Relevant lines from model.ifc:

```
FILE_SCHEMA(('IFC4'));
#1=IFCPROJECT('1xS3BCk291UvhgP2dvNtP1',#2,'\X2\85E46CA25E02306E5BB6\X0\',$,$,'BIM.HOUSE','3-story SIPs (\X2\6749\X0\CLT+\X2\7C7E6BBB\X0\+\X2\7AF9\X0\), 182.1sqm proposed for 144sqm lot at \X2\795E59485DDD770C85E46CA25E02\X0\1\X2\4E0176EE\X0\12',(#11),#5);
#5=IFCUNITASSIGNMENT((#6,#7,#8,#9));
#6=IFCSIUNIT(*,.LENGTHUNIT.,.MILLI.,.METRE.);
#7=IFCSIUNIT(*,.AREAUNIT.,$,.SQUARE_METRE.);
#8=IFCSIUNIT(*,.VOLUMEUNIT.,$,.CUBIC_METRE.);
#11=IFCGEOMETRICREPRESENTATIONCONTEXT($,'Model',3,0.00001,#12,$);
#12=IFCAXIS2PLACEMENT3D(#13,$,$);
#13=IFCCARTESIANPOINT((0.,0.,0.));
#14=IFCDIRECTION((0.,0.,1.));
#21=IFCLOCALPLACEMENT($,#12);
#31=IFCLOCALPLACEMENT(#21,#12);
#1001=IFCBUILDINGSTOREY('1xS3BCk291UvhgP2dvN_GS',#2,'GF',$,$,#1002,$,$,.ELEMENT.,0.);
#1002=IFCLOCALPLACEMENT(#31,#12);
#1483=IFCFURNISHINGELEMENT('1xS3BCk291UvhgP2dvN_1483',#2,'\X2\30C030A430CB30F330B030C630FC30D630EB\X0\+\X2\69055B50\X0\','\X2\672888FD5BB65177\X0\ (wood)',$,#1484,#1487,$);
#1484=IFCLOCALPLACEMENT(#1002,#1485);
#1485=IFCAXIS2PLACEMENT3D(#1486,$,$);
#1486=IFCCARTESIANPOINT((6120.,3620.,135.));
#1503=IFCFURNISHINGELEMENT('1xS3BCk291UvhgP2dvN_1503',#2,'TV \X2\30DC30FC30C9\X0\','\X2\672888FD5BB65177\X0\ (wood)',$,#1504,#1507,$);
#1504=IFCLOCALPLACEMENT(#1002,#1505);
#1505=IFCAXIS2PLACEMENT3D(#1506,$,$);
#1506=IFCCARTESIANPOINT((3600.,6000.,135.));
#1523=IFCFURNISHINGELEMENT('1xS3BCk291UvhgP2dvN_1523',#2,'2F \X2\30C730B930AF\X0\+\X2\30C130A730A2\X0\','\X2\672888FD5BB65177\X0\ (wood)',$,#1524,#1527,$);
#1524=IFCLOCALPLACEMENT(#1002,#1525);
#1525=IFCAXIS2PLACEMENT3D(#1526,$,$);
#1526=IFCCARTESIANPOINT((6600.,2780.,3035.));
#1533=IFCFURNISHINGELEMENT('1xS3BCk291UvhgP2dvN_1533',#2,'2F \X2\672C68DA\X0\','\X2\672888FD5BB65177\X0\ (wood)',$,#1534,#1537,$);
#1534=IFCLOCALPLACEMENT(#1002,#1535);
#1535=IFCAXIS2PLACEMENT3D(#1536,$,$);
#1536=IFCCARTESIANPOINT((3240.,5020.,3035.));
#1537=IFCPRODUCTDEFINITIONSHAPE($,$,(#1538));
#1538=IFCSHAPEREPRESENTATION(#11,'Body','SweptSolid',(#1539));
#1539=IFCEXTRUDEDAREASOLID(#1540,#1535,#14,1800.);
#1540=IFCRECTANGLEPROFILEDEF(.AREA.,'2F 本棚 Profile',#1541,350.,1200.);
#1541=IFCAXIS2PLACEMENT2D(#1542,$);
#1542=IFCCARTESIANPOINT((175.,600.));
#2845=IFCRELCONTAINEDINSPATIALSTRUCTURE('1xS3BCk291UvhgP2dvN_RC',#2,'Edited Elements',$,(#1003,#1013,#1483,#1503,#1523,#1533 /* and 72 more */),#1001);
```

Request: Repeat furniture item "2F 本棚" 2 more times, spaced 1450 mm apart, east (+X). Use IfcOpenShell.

```python
import numpy as np
import ifcopenshell
import ifcopenshell.api.geometry
import ifcopenshell.api.root
import ifcopenshell.util.element
import ifcopenshell.util.placement
import ifcopenshell.util.unit

model = ifcopenshell.open("model.ifc")
unit_scale = ifcopenshell.util.unit.calculate_unit_scale(model)


def reuse_history(source, copy):
    """copy_class also copies each property set's owner history, people and application; keep the originals."""
    for rel in copy.IsDefinedBy:
        if rel.is_a("IfcRelDefinesByProperties") and (history := rel.RelatingPropertyDefinition.OwnerHistory):
            rel.RelatingPropertyDefinition.OwnerHistory = source.OwnerHistory
            ifcopenshell.util.element.remove_deep2(model, history)


source = model.by_guid("1xS3BCk291UvhgP2dvN_1533")
base = ifcopenshell.util.placement.get_local_placement(source.ObjectPlacement)
step = np.array([1.0, 0.0, 0.0]) * 1.45 / unit_scale

for i in range(1, 3):
    copy = ifcopenshell.api.root.copy_class(model, product=source)
    copy.Representation = ifcopenshell.util.element.copy_deep(
        model, source.Representation, exclude=["IfcGeometricRepresentationContext", "IfcRepresentationMap"]
    )
    reuse_history(source, copy)
    matrix = base.copy()
    matrix[:3, 3] += i * step
    print("added at", matrix[:3, 3].round(3) + 0.0)
    ifcopenshell.api.geometry.edit_object_placement(model, product=copy, matrix=matrix, is_si=False)

model.write("model_edited.ifc")
```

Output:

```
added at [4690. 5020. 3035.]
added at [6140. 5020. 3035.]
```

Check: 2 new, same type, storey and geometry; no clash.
